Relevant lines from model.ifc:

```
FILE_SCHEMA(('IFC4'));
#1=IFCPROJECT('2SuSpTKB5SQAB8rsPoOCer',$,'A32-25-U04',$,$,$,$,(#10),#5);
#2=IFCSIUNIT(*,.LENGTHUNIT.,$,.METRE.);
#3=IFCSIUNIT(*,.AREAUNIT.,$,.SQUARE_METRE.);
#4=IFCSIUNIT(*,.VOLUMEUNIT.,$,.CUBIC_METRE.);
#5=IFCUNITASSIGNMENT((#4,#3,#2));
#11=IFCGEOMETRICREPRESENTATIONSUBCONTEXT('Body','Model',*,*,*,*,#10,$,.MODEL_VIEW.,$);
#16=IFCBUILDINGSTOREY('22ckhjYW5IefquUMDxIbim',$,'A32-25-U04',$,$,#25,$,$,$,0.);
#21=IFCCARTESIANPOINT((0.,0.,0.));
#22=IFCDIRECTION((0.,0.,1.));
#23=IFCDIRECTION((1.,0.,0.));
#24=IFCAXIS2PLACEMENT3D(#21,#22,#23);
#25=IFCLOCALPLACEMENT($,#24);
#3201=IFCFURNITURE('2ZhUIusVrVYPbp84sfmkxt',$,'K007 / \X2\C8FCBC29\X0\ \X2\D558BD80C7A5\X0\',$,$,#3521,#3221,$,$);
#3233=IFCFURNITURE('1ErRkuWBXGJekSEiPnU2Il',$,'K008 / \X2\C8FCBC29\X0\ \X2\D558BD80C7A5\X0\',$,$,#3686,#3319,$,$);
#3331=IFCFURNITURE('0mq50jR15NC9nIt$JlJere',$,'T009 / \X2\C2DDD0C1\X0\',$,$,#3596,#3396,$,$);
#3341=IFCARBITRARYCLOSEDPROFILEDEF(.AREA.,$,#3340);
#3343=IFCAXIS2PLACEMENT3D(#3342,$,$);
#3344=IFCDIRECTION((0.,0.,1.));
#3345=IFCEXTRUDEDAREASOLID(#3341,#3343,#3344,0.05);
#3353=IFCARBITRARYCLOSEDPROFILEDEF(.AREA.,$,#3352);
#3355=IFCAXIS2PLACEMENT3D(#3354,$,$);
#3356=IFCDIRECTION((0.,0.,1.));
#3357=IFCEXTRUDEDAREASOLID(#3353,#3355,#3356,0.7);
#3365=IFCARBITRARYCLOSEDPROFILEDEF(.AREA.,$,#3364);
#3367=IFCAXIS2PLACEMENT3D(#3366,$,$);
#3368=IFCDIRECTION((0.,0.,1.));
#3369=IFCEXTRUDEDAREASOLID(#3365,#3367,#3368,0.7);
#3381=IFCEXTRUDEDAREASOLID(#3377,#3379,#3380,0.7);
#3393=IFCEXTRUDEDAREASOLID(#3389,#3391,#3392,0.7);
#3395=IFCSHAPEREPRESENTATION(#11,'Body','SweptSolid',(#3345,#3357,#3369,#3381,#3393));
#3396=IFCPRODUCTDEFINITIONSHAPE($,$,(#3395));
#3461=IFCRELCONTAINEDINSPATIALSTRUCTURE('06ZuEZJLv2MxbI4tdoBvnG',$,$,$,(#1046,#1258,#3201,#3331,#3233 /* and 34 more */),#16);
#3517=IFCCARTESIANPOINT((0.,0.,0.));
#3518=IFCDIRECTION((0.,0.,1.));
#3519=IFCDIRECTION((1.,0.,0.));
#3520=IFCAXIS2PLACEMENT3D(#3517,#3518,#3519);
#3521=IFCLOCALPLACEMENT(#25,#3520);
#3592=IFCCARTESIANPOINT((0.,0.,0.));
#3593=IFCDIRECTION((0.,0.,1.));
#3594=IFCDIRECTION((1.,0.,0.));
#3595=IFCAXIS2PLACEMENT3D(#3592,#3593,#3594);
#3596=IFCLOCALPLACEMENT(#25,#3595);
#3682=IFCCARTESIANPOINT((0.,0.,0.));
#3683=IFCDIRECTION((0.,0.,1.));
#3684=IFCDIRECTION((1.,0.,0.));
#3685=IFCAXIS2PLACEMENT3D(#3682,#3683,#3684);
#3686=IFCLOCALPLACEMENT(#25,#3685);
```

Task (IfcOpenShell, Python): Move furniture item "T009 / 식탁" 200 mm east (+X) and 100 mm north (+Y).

```python
import ifcopenshell
import ifcopenshell.api.geometry
import ifcopenshell.util.placement
import ifcopenshell.util.unit

model = ifcopenshell.open("model.ifc")
unit_scale = ifcopenshell.util.unit.calculate_unit_scale(model)

item = model.by_id(3331)
matrix = ifcopenshell.util.placement.get_local_placement(item.ObjectPlacement)
matrix[0, 3] += 0.2 / unit_scale
matrix[1, 3] += 0.1 / unit_scale
ifcopenshell.api.geometry.edit_object_placement(model, product=item, matrix=matrix, is_si=False)

print(ifcopenshell.util.placement.get_local_placement(item.ObjectPlacement).round(3) + 0.0)

model.write("model_edited.ifc")
```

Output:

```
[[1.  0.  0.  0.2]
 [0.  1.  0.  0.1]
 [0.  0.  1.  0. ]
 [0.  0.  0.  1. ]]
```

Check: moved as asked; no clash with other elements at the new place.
